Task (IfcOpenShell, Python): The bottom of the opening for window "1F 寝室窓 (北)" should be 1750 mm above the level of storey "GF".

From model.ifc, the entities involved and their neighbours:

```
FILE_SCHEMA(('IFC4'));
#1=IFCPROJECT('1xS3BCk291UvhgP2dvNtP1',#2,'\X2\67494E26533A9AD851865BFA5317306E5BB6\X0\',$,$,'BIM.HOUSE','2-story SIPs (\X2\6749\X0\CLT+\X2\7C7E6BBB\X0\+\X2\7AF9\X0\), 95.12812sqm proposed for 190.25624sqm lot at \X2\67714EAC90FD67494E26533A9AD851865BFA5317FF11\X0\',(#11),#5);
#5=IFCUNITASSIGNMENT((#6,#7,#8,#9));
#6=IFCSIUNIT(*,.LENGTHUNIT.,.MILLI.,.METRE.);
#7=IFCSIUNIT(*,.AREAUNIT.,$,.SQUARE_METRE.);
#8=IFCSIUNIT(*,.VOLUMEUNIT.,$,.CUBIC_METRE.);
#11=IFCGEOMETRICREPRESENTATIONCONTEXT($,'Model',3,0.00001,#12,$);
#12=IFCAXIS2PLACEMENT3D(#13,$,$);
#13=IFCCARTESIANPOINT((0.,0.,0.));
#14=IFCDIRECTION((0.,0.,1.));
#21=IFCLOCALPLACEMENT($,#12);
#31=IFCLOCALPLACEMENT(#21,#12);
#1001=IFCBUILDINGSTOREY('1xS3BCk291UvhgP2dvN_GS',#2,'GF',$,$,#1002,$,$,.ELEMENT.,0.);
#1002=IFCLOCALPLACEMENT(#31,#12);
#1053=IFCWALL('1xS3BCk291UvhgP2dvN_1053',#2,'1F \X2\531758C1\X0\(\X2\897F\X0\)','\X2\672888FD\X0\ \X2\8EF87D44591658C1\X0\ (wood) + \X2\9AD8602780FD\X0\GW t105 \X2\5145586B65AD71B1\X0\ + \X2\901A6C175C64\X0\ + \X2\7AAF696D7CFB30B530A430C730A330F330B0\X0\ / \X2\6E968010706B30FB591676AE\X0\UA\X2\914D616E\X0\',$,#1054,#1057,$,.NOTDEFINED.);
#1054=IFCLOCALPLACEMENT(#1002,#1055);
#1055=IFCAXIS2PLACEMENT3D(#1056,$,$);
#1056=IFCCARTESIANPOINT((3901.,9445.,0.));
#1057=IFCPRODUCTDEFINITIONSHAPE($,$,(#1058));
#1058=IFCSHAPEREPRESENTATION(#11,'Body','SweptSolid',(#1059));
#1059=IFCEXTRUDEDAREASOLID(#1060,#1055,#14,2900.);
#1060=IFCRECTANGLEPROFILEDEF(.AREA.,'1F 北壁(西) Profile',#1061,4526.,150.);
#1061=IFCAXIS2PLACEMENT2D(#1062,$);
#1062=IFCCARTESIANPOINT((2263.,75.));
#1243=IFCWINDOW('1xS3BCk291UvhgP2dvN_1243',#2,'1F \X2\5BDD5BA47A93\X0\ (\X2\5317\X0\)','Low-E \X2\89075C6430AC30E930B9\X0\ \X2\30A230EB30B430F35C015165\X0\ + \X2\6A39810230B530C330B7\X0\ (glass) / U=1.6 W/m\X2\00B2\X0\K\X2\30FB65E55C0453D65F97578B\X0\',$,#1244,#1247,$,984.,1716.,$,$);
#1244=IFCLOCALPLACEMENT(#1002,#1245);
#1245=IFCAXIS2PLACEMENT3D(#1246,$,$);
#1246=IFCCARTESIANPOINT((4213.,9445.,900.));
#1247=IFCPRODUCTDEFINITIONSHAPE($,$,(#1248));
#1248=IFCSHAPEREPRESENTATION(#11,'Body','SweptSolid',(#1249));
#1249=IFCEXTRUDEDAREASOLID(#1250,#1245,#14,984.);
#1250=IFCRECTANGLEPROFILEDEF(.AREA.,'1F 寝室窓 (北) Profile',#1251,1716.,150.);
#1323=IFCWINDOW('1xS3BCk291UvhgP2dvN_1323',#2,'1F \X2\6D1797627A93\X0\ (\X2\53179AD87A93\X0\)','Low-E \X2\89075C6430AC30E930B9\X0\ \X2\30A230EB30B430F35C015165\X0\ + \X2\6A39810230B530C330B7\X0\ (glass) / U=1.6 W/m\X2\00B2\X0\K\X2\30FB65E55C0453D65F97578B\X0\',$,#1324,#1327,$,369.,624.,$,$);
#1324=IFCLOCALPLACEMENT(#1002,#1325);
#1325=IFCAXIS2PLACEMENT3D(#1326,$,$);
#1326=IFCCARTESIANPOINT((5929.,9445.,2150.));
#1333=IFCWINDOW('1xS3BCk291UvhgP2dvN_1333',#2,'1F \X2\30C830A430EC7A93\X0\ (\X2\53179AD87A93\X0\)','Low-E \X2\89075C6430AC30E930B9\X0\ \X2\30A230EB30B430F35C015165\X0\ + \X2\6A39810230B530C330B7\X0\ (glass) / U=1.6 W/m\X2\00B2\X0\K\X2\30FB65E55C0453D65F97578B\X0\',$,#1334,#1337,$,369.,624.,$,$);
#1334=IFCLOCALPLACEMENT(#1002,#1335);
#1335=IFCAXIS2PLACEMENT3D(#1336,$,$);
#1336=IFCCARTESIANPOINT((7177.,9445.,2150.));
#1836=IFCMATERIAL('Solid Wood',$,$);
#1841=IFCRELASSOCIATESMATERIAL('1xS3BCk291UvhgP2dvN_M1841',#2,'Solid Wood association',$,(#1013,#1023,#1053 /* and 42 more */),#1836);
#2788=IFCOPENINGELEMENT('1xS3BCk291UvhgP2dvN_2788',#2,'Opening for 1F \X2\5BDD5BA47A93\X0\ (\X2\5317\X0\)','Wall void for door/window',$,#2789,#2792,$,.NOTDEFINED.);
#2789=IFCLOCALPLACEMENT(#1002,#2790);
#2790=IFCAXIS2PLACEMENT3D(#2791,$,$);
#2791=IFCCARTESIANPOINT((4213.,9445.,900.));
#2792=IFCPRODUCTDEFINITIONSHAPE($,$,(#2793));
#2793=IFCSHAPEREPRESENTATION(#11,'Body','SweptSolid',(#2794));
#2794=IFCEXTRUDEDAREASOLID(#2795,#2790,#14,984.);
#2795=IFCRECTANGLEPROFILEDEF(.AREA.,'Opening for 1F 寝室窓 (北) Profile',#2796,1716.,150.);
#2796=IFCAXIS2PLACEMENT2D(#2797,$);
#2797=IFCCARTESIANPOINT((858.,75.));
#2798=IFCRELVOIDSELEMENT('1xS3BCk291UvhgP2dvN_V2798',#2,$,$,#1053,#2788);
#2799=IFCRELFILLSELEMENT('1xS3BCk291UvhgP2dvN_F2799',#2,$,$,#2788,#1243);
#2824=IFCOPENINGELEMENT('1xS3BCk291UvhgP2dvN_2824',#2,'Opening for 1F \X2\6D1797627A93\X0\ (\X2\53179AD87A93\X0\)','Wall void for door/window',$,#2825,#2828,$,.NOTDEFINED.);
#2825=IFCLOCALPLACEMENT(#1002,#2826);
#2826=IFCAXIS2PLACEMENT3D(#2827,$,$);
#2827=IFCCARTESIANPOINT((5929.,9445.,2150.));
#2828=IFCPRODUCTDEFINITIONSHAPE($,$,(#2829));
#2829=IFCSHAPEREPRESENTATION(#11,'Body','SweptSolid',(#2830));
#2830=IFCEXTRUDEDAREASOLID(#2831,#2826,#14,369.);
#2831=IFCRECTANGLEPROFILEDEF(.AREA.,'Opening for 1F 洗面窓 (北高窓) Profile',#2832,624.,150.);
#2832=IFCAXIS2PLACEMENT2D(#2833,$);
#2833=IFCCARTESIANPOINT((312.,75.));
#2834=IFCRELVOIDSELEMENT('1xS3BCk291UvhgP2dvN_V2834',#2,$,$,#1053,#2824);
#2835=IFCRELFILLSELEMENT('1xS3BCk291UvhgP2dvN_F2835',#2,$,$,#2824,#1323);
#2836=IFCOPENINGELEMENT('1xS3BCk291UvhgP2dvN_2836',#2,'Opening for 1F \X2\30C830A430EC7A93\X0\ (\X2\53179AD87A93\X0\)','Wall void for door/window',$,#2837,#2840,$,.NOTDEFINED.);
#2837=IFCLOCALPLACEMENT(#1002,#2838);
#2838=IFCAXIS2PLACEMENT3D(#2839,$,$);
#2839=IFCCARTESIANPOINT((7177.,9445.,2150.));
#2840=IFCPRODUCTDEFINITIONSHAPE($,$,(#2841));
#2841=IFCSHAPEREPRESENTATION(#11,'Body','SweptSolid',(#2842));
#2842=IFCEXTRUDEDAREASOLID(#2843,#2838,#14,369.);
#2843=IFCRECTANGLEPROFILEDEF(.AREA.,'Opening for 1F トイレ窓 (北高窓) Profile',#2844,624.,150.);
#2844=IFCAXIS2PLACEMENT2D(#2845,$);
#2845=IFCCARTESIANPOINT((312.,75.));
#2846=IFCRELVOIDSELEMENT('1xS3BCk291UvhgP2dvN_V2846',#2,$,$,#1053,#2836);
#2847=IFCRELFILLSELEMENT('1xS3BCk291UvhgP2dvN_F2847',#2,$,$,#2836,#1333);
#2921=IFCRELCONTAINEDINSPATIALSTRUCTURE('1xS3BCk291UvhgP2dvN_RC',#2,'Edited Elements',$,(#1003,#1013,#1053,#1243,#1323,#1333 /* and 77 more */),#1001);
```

```python
import numpy as np
import ifcopenshell
import ifcopenshell.api.geometry
import ifcopenshell.geom
import ifcopenshell.util.element
import ifcopenshell.util.placement
import ifcopenshell.util.shape
import ifcopenshell.util.unit

model = ifcopenshell.open("model.ifc")
unit_scale = ifcopenshell.util.unit.calculate_unit_scale(model)

window = model.by_guid("1xS3BCk291UvhgP2dvN_1243")
opening = window.FillsVoids[0].RelatingOpeningElement
storey = ifcopenshell.util.element.get_container(window, ifc_class="IfcBuildingStorey")
level = ifcopenshell.util.placement.get_local_placement(storey.ObjectPlacement)[2, 3]

# The opening's origin need not be at the sill, so measure its lowest point.
shape = ifcopenshell.geom.create_shape(ifcopenshell.geom.settings(), opening)
bottom = ifcopenshell.util.shape.get_shape_bottom_elevation(shape, shape.geometry) / unit_scale
dz = level + 1.75 / unit_scale - bottom

shift = np.array([0.0, 0.0, dz])
# The window is not placed relative to its opening, so move both.
for product in (opening, window):
    matrix = ifcopenshell.util.placement.get_local_placement(product.ObjectPlacement)
    matrix[:3, 3] += shift
    ifcopenshell.api.geometry.edit_object_placement(model, product=product, matrix=matrix, is_si=False)

print(f"moved by {dz * unit_scale:+.3f} m")

model.write("model_v2.ifc")
```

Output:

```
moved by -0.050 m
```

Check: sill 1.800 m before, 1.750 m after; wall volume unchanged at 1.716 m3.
